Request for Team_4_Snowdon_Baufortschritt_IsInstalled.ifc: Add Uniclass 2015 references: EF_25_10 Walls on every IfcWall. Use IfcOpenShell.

First a look at what the model holds.

```python
import ifcopenshell

model = ifcopenshell.open("Team_4_Snowdon_Baufortschritt_IsInstalled.ifc")
print(model.schema)
print("classifications:", [c.Name for c in model.by_type("IfcClassification")])
for ifc_class in ("IfcDoor", "IfcRoof", "IfcStair", "IfcWall", "IfcWindow"):
    print(ifc_class, len(model.by_type(ifc_class)))
```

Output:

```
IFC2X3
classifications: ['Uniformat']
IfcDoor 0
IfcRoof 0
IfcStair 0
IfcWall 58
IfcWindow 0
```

```python
import ifcopenshell
import ifcopenshell.api.classification

model = ifcopenshell.open("Team_4_Snowdon_Baufortschritt_IsInstalled.ifc")

# IFC2X3 requires Source and Edition and has no link from the project to the system.
system = model.create_entity("IfcClassification", Source="NBS", Edition="2015", Name="Uniclass 2015")

codes = {
    "IfcWall": ("EF_25_10", "Walls"),
}
for ifc_class, (code, name) in codes.items():
    products = model.by_type(ifc_class)
    ifcopenshell.api.classification.add_reference(
        model, products=products, classification=system, identification=code, name=name
    )
    print(code, len(products))

model.write("Team_4_Snowdon_Baufortschritt_IsInstalled_updated.ifc")
```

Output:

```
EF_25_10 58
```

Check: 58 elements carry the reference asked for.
